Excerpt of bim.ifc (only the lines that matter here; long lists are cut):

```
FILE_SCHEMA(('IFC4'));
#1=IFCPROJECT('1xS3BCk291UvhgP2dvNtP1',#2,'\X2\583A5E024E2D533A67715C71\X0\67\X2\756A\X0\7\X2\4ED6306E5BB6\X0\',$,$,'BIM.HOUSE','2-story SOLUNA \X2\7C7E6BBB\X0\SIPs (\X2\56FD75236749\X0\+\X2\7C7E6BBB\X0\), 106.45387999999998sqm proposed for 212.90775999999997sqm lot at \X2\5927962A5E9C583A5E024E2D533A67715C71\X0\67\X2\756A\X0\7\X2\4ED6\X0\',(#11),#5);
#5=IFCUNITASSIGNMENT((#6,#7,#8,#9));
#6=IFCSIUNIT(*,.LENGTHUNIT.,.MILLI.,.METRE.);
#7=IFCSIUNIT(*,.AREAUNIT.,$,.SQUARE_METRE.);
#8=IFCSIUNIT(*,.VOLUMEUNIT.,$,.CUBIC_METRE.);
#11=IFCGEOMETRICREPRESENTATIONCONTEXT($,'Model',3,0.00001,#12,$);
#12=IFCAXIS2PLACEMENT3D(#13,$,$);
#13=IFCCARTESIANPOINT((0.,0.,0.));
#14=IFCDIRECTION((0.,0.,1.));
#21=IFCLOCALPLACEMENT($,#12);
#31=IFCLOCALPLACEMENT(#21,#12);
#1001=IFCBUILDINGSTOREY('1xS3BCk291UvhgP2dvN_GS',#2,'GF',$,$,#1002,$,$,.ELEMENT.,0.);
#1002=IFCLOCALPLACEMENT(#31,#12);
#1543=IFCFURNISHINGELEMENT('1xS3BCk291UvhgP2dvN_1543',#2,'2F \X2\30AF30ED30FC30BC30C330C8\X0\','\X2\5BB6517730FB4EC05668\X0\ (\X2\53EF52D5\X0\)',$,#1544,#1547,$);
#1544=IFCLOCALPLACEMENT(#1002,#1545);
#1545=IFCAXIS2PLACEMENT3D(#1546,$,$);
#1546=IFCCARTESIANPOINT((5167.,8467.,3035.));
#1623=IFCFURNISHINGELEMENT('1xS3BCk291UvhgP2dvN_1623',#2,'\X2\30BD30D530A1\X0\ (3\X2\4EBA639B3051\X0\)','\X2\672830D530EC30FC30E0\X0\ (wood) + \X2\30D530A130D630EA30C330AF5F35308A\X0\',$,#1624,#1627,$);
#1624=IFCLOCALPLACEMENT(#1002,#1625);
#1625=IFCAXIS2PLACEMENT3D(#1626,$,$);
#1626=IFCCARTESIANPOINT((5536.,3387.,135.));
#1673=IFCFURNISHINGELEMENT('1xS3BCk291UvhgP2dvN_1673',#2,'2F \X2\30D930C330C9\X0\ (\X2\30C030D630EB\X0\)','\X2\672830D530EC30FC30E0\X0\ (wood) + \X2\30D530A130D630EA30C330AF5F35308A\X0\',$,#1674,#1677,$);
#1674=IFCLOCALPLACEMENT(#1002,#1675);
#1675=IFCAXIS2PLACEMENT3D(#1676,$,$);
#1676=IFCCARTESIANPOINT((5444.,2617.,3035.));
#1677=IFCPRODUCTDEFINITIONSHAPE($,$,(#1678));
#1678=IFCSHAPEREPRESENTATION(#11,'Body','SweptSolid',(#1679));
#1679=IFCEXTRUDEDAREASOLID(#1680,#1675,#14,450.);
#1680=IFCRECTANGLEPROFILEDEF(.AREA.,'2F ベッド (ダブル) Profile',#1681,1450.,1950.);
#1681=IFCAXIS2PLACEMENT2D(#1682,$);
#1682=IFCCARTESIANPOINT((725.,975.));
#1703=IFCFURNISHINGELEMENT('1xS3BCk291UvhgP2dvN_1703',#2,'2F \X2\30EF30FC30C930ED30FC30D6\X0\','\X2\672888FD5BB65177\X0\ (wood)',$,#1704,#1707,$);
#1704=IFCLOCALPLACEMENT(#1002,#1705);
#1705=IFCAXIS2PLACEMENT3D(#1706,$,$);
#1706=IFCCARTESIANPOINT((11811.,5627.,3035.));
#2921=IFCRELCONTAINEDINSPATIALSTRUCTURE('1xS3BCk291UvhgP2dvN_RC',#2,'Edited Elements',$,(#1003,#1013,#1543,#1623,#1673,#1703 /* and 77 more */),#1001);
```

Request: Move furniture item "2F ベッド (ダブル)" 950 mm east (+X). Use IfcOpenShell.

```python
import ifcopenshell
import ifcopenshell.api.geometry
import ifcopenshell.util.placement
import ifcopenshell.util.unit

model = ifcopenshell.open("bim.ifc")
unit_scale = ifcopenshell.util.unit.calculate_unit_scale(model)

item = model.by_guid("1xS3BCk291UvhgP2dvN_1673")
matrix = ifcopenshell.util.placement.get_local_placement(item.ObjectPlacement)
matrix[0, 3] += 0.95 / unit_scale
ifcopenshell.api.geometry.edit_object_placement(model, product=item, matrix=matrix, is_si=False)

print(ifcopenshell.util.placement.get_local_placement(item.ObjectPlacement).round(3) + 0.0)

model.write("bim_rev.ifc")
```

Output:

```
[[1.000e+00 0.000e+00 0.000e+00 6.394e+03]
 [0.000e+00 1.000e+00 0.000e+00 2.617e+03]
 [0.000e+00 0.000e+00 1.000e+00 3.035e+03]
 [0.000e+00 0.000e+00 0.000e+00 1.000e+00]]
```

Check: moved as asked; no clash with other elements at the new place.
